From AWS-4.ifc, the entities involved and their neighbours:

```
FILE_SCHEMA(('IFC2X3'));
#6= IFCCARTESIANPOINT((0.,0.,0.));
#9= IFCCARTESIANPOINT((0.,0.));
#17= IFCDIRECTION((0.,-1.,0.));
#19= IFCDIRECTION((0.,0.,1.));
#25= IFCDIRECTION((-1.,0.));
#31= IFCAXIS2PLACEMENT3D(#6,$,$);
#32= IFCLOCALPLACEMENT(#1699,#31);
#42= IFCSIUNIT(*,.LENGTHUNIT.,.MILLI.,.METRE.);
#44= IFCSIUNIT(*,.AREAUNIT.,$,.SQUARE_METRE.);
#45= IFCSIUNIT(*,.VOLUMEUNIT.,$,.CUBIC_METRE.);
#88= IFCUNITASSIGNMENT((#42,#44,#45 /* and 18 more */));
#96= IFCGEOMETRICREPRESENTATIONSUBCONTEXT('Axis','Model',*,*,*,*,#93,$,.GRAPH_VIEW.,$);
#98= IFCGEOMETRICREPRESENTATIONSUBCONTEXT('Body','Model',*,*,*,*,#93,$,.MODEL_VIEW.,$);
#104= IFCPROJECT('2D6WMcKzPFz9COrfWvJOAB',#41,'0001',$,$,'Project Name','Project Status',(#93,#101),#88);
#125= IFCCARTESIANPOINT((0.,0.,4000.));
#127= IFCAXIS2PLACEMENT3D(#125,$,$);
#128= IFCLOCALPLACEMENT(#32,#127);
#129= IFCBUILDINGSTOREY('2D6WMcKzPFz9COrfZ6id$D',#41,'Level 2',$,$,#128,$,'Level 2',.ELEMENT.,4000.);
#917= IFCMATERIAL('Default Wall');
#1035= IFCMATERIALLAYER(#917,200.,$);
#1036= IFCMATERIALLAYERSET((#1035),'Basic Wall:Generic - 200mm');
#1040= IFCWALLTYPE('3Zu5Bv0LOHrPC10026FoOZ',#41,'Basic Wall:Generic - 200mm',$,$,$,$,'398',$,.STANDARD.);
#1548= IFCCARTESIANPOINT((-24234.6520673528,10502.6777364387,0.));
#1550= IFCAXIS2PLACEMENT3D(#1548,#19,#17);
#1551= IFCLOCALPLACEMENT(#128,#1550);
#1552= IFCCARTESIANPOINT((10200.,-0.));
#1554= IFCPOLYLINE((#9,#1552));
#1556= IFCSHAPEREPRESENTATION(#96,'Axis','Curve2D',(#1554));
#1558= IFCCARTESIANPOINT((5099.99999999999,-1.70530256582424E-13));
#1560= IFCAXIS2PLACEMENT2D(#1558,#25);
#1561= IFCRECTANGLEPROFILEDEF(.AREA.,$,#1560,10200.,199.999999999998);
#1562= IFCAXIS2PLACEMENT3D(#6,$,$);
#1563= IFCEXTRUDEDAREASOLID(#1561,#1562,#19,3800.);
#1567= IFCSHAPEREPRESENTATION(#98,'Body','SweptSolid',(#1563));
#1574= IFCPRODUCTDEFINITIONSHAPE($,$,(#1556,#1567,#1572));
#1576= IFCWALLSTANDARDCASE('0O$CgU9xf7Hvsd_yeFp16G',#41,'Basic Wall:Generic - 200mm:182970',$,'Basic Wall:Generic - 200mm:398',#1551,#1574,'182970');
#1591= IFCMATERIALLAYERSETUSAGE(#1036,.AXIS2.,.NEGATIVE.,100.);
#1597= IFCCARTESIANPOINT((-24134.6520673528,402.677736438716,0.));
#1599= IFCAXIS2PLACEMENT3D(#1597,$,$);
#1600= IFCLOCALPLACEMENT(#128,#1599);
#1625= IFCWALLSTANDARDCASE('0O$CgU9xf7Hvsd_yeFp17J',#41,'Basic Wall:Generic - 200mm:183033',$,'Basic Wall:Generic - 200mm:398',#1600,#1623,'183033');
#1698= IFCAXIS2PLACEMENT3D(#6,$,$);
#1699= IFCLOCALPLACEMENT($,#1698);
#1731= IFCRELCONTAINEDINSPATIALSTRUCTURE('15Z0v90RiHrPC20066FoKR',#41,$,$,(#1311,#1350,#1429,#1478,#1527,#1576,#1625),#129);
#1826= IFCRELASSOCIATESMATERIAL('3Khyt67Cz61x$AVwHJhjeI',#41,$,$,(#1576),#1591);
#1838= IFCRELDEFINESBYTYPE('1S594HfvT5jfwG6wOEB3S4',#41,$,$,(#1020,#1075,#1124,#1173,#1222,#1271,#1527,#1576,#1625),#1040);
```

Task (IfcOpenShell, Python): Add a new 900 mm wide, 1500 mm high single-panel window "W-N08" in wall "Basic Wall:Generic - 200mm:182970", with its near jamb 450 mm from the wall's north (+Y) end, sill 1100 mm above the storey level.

```python
import numpy as np
import ifcopenshell
import ifcopenshell.api.feature
import ifcopenshell.api.geometry
import ifcopenshell.api.root
import ifcopenshell.api.spatial
import ifcopenshell.api.type
import ifcopenshell.geom
import ifcopenshell.util.element
import ifcopenshell.util.placement
import ifcopenshell.util.representation
import ifcopenshell.util.shape
import ifcopenshell.util.unit

model = ifcopenshell.open("AWS-4.ifc")
unit_scale = ifcopenshell.util.unit.calculate_unit_scale(model)
settings = ifcopenshell.geom.settings()


def volume(element):
    """Net volume in cubic metres, openings subtracted."""
    shape = ifcopenshell.geom.create_shape(settings, element)
    return ifcopenshell.util.shape.get_volume(shape.geometry)


wall = model.by_id(1576)
storey = ifcopenshell.util.element.get_container(wall, ifc_class="IfcBuildingStorey")
context = ifcopenshell.util.representation.get_context(model, "Model", "Body", "MODEL_VIEW")
before = volume(wall)

width, height, from_end, sill = 0.9, 1.5, 0.45, 1.1  # metres

# The wall runs along its own X axis, and the end named is its -X end.
wall_shape = ifcopenshell.geom.create_shape(settings, wall)
x, y, z = ifcopenshell.util.shape.get_vertices(wall_shape.geometry).T
start = x.min() + from_end
face, thickness = float(y.min()), float(y.max() - y.min())
wall_matrix = ifcopenshell.util.placement.get_local_placement(wall.ObjectPlacement)
level = ifcopenshell.util.placement.get_local_placement(storey.ObjectPlacement)[2, 3]


def in_wall(x, y):
    """Placement at x, y metres in the wall's axes, at sill height."""
    matrix = wall_matrix.copy()
    matrix[:, 3] = wall_matrix @ np.array([x / unit_scale, y / unit_scale, 0.0, 1.0])
    matrix[2, 3] = level + sill / unit_scale
    return matrix


# Opening: a box that overshoots both wall faces by 50 mm.
opening = ifcopenshell.api.root.create_entity(model, ifc_class="IfcOpeningElement")
box = ifcopenshell.api.geometry.add_wall_representation(
    model, context=context, length=width, height=height, thickness=thickness + 0.1
)
ifcopenshell.api.geometry.assign_representation(model, product=opening, representation=box)
ifcopenshell.api.geometry.edit_object_placement(model, product=opening, matrix=in_wall(start, face - 0.05), is_si=False)
ifcopenshell.api.feature.add_feature(model, feature=opening, element=wall)

window = ifcopenshell.api.root.create_entity(model, ifc_class="IfcWindow", name="W-N08")
window.OverallWidth, window.OverallHeight = width / unit_scale, height / unit_scale
body = ifcopenshell.api.geometry.add_window_representation(
    model,
    context=context,
    overall_width=window.OverallWidth,
    overall_height=window.OverallHeight,
    partition_type="SINGLE_PANEL",
)
ifcopenshell.api.geometry.assign_representation(model, product=window, representation=body)
ifcopenshell.api.spatial.assign_container(model, products=[window], relating_structure=storey)
fills = ifcopenshell.api.feature.add_filling(model, opening=opening, element=window)
fills.OwnerHistory = window.OwnerHistory  # required in IFC2X3

# IFC2X3 keeps the operation on the window style.
style = ifcopenshell.api.root.create_entity(model, ifc_class="IfcWindowStyle", name="W-N08")
style.OperationType, style.ConstructionType = "SINGLE_PANEL", "NOTDEFINED"
style.ParameterTakesPrecedence = style.Sizeable = False
ifcopenshell.api.type.assign_type(model, related_objects=[window], relating_type=style)

# Centre the window in the wall's thickness.
ifcopenshell.api.geometry.edit_object_placement(model, product=window, matrix=in_wall(start, face), is_si=False)
window_shape = ifcopenshell.geom.create_shape(settings, window)
depth = ifcopenshell.util.shape.get_vertices(window_shape.geometry)[:, 1]
offset = face + thickness / 2 - (depth.min() + depth.max()) / 2
ifcopenshell.api.geometry.edit_object_placement(model, product=window, matrix=in_wall(start, offset), is_si=False)

after = volume(wall)

print(f"wall volume {before:.3f} -> {after:.3f} m3")

model.write("AWS-4_rev.ifc")
```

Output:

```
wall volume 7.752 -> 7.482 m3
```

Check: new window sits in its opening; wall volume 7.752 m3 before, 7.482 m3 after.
